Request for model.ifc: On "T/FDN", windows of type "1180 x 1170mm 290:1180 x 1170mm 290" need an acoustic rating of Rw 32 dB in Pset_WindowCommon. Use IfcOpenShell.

First a look at what the model holds.

```python
import ifcopenshell
import ifcopenshell.util.element

model = ifcopenshell.open("model.ifc")
print(model.schema)
storey = next(s for s in model.by_type("IfcBuildingStorey") if s.Name == "T/FDN")
windows = [e for e in ifcopenshell.util.element.get_decomposition(storey) if e.is_a("IfcWindow")]
seen = {}
for e in windows:
    element_type = ifcopenshell.util.element.get_type(e)
    key = (element_type.Name if element_type != e and element_type else None, ifcopenshell.util.element.get_pset(e, "Pset_WindowCommon", "AcousticRating"))
    seen[key] = seen.get(key, 0) + 1
for (name, value), count in sorted(seen.items(), key=str):
    print(count, "x", name, "|", value)
```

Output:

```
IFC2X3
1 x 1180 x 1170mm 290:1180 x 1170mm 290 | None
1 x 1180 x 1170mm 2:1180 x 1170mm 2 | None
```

```python
import ifcopenshell
import ifcopenshell.api.pset
import ifcopenshell.util.element

model = ifcopenshell.open("model.ifc")

storey = next(s for s in model.by_type("IfcBuildingStorey") if s.Name == "T/FDN")
windows = [e for e in ifcopenshell.util.element.get_decomposition(storey) if e.is_a("IfcWindow")]

count = 0
for e in windows:
    element_type = ifcopenshell.util.element.get_type(e)
    if element_type in (None, e) or element_type.Name != "1180 x 1170mm 290:1180 x 1170mm 290":
        continue
    # add_pset returns the element's existing set when there is one.
    pset = ifcopenshell.api.pset.add_pset(model, product=e, name="Pset_WindowCommon")
    ifcopenshell.api.pset.edit_pset(model, pset=pset, properties={"AcousticRating": "Rw 32 dB"})
    count += 1

print(count, "windows updated")

model.write("model_updated.ifc")
```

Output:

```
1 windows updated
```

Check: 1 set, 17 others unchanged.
